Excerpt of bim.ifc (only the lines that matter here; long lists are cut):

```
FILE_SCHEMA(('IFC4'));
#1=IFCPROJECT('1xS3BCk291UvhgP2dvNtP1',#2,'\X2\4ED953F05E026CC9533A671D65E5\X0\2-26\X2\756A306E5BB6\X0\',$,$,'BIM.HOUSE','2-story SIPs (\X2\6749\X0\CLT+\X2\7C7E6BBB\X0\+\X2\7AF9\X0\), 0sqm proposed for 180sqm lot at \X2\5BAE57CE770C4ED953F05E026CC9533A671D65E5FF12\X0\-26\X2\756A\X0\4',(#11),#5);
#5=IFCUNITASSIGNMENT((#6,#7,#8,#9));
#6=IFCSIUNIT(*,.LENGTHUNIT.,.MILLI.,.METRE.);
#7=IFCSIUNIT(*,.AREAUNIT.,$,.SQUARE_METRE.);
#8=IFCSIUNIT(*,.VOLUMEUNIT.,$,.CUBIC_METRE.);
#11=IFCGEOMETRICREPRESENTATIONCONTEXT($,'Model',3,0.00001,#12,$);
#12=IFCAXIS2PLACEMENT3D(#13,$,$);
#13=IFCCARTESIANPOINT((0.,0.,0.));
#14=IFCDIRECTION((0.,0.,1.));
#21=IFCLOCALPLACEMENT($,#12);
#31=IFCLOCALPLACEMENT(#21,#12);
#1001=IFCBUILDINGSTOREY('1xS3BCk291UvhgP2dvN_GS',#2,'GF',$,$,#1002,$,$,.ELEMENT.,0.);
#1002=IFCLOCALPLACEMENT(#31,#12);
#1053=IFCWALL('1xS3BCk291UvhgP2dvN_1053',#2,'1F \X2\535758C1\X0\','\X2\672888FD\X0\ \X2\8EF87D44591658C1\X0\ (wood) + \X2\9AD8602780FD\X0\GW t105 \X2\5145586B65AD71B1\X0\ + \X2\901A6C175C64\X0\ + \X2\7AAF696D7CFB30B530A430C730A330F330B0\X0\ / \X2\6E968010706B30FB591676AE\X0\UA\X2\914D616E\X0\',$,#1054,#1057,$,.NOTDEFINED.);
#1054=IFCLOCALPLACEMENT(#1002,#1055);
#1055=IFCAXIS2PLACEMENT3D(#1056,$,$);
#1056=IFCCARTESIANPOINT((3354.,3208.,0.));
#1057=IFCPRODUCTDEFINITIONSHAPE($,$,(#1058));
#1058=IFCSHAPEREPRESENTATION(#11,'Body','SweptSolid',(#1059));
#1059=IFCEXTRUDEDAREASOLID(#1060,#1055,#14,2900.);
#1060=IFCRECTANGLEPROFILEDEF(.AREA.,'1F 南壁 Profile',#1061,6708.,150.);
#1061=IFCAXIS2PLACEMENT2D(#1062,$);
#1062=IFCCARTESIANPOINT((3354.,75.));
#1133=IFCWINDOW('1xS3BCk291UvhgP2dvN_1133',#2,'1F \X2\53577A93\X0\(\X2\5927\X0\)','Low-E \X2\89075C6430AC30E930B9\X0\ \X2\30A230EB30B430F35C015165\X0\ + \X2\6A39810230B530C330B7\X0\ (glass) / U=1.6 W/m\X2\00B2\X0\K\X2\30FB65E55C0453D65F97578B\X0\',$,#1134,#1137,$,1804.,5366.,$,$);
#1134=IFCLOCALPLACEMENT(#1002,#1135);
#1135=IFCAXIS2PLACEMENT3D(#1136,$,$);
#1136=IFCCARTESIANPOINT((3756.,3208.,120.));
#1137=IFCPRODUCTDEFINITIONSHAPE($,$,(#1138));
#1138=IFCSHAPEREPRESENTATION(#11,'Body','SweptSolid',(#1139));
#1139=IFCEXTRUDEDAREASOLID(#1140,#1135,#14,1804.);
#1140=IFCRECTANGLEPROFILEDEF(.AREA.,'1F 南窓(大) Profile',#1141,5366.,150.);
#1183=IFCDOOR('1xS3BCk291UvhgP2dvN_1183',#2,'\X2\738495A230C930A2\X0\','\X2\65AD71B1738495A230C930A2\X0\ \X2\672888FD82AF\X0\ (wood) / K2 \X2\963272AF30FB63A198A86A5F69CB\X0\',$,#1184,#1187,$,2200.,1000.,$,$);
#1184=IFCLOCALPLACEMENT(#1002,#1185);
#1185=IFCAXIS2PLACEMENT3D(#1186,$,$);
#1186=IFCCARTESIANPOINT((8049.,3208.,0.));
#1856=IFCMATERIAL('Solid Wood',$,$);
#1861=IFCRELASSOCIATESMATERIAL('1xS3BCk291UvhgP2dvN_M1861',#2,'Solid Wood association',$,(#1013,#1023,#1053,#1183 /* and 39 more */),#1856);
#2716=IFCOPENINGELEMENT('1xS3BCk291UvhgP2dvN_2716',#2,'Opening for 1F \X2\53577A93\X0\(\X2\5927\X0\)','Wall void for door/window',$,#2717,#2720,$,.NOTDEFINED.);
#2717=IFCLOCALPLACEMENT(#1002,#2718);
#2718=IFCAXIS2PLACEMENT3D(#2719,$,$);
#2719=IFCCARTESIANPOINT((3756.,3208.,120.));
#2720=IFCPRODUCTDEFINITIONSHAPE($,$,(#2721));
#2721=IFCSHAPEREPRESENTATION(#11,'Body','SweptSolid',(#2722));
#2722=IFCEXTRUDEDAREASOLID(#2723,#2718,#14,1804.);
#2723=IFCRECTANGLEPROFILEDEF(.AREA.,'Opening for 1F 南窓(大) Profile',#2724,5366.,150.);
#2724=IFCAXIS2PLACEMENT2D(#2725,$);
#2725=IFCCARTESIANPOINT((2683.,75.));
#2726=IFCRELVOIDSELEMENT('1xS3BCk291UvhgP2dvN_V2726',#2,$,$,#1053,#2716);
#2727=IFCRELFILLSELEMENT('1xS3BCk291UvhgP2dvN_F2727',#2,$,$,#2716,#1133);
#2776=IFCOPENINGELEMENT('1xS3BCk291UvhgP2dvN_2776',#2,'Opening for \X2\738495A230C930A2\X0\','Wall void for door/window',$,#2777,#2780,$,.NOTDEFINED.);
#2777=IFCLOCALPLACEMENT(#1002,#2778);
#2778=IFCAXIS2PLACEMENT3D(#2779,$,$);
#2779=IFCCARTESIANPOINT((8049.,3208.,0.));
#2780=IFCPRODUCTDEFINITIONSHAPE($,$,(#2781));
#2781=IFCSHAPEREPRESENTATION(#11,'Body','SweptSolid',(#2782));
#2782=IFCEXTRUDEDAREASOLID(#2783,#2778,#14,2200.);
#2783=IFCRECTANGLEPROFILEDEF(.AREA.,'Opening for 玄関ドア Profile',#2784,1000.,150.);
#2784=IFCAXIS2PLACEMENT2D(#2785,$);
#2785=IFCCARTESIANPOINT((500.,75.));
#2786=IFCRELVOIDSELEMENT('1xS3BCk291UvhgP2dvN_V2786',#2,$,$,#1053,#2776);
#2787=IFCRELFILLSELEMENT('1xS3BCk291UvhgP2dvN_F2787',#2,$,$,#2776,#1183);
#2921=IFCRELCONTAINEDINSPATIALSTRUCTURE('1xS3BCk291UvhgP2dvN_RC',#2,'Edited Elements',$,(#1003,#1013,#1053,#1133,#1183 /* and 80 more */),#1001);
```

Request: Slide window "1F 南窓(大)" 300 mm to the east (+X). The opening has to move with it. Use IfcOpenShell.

```python
import ifcopenshell
import ifcopenshell.api.geometry
import ifcopenshell.util.placement
import ifcopenshell.util.unit

model = ifcopenshell.open("bim.ifc")
unit_scale = ifcopenshell.util.unit.calculate_unit_scale(model)

window = model.by_guid("1xS3BCk291UvhgP2dvN_1133")
opening = window.FillsVoids[0].RelatingOpeningElement
wall = opening.VoidsElements[0].RelatingBuildingElement

wall_matrix = ifcopenshell.util.placement.get_local_placement(wall.ObjectPlacement)
shift = wall_matrix[:3, 0] * 0.3 / unit_scale
before = ifcopenshell.util.placement.get_local_placement(window.ObjectPlacement)[:3, 3].copy()

# The window is not placed relative to its opening, so move both.
for product in (opening, window):
    matrix = ifcopenshell.util.placement.get_local_placement(product.ObjectPlacement)
    matrix[:3, 3] += shift
    ifcopenshell.api.geometry.edit_object_placement(model, product=product, matrix=matrix, is_si=False)

after = ifcopenshell.util.placement.get_local_placement(window.ObjectPlacement)[:3, 3]
print("window moved by", (after - before).round(3) + 0.0)

model.write("bim_rev.ifc")
```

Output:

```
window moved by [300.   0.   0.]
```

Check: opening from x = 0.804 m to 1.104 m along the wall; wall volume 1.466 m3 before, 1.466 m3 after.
